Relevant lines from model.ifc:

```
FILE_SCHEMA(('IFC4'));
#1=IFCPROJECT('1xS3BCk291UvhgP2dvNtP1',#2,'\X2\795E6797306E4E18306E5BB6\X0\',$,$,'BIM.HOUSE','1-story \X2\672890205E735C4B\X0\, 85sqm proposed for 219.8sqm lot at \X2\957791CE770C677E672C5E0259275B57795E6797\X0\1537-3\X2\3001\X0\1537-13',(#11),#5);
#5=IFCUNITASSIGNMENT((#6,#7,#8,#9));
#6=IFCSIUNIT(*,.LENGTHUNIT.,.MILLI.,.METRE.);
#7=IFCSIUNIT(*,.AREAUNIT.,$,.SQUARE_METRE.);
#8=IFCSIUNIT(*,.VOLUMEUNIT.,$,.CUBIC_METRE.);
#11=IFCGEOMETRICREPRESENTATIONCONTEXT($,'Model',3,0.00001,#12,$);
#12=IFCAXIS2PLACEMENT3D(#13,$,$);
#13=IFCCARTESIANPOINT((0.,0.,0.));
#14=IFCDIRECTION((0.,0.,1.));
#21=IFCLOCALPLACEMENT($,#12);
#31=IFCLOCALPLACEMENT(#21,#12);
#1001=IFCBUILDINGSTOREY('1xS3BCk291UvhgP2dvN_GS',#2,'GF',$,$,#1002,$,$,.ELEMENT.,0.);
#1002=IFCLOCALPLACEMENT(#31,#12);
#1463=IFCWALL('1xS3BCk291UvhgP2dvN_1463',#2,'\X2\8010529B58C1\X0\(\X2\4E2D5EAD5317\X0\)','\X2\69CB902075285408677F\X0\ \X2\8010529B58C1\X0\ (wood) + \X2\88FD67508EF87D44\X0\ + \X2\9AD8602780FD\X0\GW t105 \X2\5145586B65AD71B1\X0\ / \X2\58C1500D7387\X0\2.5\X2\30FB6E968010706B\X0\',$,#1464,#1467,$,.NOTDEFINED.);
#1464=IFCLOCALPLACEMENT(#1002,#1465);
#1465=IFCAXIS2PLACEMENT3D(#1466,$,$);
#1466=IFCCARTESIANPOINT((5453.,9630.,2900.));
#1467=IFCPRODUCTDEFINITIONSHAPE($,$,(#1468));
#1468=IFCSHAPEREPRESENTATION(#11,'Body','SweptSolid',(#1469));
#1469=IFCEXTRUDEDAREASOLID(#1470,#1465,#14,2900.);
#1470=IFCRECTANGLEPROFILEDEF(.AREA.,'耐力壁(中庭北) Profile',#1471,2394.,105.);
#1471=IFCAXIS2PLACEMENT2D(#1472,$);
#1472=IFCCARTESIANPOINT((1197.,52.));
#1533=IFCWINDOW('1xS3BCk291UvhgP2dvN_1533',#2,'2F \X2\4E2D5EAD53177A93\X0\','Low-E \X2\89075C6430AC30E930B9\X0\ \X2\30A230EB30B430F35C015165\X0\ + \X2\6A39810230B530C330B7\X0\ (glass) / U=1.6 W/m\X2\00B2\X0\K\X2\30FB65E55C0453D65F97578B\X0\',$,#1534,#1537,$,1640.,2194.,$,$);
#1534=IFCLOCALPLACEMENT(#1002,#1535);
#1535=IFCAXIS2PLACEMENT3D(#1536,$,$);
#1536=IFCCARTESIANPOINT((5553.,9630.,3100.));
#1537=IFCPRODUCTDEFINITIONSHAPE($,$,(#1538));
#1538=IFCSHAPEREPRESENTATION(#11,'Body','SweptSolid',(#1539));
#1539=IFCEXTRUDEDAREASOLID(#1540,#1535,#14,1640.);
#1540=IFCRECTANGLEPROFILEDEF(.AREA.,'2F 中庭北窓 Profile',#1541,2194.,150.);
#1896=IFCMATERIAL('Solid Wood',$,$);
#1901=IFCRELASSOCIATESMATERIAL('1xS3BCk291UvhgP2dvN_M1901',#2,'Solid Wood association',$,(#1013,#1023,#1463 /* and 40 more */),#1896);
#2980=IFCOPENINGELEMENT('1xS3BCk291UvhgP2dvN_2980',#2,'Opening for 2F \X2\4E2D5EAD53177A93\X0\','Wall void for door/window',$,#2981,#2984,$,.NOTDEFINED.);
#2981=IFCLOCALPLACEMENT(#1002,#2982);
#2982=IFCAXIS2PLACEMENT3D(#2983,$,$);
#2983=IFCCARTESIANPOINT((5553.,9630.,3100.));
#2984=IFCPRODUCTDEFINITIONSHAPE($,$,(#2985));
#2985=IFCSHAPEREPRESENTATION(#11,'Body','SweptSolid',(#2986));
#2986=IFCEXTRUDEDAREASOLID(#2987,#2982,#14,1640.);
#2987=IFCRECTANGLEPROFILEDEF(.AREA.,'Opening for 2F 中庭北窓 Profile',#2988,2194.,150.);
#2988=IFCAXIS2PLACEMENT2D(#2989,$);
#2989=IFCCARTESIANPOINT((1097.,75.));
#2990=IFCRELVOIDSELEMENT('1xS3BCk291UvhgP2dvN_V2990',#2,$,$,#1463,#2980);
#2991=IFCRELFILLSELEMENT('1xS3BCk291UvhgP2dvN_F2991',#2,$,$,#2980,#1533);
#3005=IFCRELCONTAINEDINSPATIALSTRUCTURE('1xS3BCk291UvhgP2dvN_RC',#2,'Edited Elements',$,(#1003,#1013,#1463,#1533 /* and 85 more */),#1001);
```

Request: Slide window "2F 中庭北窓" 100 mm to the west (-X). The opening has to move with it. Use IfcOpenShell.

```python
import ifcopenshell
import ifcopenshell.api.geometry
import ifcopenshell.util.placement

model = ifcopenshell.open("model.ifc")

window = model.by_guid("1xS3BCk291UvhgP2dvN_1533")
opening = window.FillsVoids[0].RelatingOpeningElement
wall = opening.VoidsElements[0].RelatingBuildingElement

wall_matrix = ifcopenshell.util.placement.get_local_placement(wall.ObjectPlacement)
shift = wall_matrix[:3, 0] * -100.0
before = ifcopenshell.util.placement.get_local_placement(window.ObjectPlacement)[:3, 3].copy()

# The window is not placed relative to its opening, so move both.
for product in (opening, window):
    matrix = ifcopenshell.util.placement.get_local_placement(product.ObjectPlacement)
    matrix[:3, 3] += shift
    ifcopenshell.api.geometry.edit_object_placement(model, product=product, matrix=matrix, is_si=False)

after = ifcopenshell.util.placement.get_local_placement(window.ObjectPlacement)[:3, 3]
print("window moved by", (after - before).round(3) + 0.0)

model.write("model_v2.ifc")
```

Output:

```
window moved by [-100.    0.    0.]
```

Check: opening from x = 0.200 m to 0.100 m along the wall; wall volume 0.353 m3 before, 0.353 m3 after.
